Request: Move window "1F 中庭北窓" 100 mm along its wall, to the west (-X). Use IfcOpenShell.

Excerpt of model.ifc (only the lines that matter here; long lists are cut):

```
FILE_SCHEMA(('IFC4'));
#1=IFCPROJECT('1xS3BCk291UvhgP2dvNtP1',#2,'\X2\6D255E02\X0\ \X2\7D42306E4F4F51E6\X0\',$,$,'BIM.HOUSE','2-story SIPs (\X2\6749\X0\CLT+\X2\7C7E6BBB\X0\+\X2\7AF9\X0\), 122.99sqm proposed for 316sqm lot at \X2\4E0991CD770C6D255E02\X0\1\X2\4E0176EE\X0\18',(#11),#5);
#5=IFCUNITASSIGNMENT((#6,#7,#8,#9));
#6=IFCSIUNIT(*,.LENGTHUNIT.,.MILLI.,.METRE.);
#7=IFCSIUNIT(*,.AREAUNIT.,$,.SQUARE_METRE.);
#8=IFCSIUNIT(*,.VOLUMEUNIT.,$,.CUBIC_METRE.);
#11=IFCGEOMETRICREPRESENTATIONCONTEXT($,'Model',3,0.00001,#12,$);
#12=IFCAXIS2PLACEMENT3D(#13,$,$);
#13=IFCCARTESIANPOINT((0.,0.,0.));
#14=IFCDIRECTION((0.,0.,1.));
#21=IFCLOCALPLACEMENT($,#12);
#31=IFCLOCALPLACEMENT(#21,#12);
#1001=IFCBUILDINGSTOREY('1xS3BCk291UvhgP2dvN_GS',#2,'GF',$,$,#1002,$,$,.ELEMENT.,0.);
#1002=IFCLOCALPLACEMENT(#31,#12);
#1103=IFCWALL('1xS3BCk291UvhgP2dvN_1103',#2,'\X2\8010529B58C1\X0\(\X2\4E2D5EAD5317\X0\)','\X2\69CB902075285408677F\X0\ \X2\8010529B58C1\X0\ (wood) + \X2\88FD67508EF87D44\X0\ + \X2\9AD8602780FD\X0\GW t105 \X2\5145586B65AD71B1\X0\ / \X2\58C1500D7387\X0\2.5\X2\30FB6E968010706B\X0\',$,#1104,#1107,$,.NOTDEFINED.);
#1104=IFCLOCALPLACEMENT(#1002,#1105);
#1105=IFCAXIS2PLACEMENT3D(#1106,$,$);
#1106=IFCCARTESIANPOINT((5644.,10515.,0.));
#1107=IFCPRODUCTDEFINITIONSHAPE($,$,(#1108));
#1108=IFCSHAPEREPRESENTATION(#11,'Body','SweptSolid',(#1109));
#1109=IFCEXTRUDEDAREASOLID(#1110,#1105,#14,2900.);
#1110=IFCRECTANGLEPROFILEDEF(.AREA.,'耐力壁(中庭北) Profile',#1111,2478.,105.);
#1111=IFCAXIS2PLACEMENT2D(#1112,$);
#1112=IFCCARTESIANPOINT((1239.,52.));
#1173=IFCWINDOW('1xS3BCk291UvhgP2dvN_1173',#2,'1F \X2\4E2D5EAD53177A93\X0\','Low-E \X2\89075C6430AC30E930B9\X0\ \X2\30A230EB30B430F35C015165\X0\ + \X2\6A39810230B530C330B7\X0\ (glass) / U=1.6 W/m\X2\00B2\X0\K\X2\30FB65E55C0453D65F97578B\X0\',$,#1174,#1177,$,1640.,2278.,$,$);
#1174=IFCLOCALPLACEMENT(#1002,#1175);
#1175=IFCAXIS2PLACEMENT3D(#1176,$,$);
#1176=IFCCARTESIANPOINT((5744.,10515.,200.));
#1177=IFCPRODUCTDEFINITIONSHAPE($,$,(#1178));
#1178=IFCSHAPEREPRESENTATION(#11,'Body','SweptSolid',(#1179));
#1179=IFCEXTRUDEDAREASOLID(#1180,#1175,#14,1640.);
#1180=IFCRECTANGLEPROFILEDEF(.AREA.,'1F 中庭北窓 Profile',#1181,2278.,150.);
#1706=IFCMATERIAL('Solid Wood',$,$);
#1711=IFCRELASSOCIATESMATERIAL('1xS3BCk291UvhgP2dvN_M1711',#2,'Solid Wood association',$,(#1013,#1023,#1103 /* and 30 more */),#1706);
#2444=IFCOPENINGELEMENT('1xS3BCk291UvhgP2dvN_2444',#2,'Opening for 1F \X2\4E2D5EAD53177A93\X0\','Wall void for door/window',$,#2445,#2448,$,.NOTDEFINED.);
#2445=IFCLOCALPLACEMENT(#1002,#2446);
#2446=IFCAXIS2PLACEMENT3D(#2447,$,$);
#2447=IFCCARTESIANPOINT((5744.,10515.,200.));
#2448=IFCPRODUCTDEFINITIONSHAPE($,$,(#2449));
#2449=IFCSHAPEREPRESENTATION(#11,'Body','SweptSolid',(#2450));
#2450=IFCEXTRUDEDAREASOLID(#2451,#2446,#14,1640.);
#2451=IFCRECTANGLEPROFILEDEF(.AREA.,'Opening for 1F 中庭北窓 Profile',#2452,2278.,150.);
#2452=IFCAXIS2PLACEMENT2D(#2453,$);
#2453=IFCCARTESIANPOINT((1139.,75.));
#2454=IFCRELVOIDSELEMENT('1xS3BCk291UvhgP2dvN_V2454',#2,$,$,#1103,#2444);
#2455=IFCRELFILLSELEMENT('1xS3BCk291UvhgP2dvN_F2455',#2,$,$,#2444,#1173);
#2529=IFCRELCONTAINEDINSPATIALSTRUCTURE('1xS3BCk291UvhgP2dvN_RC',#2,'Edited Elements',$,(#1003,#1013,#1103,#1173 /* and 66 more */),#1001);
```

```python
import ifcopenshell
import ifcopenshell.api.geometry
import ifcopenshell.util.placement
import ifcopenshell.util.unit

model = ifcopenshell.open("model.ifc")
unit_scale = ifcopenshell.util.unit.calculate_unit_scale(model)

window = model.by_guid("1xS3BCk291UvhgP2dvN_1173")
opening = window.FillsVoids[0].RelatingOpeningElement
wall = opening.VoidsElements[0].RelatingBuildingElement

wall_matrix = ifcopenshell.util.placement.get_local_placement(wall.ObjectPlacement)
shift = wall_matrix[:3, 0] * -0.1 / unit_scale
before = ifcopenshell.util.placement.get_local_placement(window.ObjectPlacement)[:3, 3].copy()

# The window is not placed relative to its opening, so move both.
for product in (opening, window):
    matrix = ifcopenshell.util.placement.get_local_placement(product.ObjectPlacement)
    matrix[:3, 3] += shift
    ifcopenshell.api.geometry.edit_object_placement(model, product=product, matrix=matrix, is_si=False)

after = ifcopenshell.util.placement.get_local_placement(window.ObjectPlacement)[:3, 3]
print("window moved by", (after - before).round(3) + 0.0)

model.write("model_rev.ifc")
```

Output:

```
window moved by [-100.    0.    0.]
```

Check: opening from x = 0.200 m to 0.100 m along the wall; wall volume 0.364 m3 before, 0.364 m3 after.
